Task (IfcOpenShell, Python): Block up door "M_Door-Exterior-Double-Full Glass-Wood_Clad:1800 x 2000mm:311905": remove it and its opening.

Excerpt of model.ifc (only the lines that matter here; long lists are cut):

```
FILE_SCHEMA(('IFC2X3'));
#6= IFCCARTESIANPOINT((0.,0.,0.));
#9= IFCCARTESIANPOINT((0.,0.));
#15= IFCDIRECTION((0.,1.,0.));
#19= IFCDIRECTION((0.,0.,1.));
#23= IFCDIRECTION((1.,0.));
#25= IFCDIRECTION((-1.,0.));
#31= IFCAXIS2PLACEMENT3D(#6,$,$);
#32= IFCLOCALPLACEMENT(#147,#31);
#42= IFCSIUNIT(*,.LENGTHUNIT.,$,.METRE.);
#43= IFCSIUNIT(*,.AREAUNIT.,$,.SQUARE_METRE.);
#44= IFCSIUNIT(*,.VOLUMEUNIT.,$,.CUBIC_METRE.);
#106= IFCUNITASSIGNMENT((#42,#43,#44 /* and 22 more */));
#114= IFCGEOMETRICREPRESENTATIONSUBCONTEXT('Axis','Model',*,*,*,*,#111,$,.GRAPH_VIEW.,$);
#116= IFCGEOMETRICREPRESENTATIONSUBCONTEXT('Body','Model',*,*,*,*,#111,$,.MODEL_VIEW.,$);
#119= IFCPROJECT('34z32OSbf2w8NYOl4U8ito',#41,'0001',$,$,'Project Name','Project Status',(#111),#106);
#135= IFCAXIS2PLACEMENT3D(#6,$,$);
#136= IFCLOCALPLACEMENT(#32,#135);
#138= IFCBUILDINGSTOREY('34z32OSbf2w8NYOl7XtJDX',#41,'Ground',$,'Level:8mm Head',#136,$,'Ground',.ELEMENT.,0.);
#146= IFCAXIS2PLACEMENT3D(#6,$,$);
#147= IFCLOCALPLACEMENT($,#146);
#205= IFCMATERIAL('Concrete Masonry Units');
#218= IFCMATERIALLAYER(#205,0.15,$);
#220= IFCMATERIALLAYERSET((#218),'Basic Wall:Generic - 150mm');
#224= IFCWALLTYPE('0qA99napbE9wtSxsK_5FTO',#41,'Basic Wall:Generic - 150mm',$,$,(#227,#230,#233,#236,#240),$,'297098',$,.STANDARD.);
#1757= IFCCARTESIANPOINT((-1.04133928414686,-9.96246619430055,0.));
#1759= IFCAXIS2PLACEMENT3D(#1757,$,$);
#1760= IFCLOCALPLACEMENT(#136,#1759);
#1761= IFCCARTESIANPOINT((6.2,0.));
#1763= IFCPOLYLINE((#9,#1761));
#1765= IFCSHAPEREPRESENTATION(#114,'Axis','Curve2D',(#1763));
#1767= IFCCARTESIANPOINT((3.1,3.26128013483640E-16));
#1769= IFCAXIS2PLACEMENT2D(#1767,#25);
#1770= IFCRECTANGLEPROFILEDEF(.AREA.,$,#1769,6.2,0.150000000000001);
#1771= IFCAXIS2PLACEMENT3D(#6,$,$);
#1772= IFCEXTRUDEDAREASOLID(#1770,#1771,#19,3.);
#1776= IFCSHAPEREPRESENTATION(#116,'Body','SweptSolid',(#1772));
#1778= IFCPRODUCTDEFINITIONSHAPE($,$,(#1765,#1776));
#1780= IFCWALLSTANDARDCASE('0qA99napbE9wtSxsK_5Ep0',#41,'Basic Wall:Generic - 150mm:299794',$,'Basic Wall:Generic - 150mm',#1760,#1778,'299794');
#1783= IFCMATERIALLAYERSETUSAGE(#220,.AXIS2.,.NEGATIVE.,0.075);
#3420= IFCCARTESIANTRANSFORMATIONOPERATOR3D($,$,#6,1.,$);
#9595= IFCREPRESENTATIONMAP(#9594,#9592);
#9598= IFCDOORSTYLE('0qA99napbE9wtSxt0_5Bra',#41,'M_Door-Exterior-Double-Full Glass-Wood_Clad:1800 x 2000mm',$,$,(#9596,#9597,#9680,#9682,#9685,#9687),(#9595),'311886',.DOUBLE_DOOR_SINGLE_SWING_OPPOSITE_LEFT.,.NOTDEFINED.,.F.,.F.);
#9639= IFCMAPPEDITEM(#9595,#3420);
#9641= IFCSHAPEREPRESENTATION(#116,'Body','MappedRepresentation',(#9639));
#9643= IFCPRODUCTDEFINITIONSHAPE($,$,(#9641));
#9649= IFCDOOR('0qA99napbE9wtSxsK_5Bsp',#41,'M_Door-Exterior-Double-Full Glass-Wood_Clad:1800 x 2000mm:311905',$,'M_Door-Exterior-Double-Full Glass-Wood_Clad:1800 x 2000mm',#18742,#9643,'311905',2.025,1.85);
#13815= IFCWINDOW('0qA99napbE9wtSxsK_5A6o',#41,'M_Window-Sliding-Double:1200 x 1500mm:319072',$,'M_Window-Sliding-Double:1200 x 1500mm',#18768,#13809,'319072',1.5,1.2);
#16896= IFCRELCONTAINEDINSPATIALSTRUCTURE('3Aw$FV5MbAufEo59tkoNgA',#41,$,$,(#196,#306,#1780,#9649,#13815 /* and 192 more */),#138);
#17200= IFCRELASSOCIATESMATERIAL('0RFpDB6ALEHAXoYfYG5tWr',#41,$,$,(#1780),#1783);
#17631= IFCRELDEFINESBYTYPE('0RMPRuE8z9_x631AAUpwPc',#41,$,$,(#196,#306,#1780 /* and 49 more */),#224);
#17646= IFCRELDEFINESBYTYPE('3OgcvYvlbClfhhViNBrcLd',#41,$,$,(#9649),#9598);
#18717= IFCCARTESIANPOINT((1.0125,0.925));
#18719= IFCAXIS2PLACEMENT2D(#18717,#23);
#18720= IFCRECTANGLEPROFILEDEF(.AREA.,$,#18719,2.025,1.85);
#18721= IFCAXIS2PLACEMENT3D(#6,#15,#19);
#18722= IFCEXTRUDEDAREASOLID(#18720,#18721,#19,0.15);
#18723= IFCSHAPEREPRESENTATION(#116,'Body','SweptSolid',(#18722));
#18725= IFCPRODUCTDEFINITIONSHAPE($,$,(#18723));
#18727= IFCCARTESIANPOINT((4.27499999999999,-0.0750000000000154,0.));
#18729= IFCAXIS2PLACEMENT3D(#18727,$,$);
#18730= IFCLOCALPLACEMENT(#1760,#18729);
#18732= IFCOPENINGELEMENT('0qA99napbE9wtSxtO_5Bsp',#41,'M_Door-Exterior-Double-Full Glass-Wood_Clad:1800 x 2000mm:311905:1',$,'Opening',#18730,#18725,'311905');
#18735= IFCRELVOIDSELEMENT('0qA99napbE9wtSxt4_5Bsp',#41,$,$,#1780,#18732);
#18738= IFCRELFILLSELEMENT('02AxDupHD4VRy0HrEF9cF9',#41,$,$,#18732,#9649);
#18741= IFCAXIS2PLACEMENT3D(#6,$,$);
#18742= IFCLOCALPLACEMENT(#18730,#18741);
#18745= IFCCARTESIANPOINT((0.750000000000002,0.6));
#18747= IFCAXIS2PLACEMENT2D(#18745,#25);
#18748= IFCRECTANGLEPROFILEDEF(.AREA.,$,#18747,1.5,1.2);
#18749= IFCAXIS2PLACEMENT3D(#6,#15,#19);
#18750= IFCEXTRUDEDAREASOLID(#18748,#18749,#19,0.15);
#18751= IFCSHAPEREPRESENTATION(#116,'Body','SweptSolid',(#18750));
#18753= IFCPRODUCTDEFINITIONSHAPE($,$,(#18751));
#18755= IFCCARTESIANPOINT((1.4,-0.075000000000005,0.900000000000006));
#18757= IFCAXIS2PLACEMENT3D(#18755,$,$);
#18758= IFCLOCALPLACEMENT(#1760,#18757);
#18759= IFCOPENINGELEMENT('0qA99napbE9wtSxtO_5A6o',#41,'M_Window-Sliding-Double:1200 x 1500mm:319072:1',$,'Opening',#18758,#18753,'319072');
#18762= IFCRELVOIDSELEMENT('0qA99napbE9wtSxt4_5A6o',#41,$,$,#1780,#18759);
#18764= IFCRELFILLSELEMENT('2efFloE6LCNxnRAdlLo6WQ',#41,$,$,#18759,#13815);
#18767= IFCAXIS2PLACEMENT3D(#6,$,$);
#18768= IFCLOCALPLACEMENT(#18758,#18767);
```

```python
import ifcopenshell
import ifcopenshell.api.feature
import ifcopenshell.api.root
import ifcopenshell.geom
import ifcopenshell.util.shape

model = ifcopenshell.open("model.ifc")
settings = ifcopenshell.geom.settings()


def volume(element):
    """Net volume in cubic metres, openings subtracted."""
    shape = ifcopenshell.geom.create_shape(settings, element)
    return ifcopenshell.util.shape.get_volume(shape.geometry)


door = model.by_guid("0qA99napbE9wtSxsK_5Bsp")
opening = door.FillsVoids[0].RelatingOpeningElement
wall = opening.VoidsElements[0].RelatingBuildingElement
before = volume(wall)

ifcopenshell.api.root.remove_product(model, product=door)
ifcopenshell.api.feature.remove_feature(model, feature=opening)

after = volume(wall)

print(f"wall volume {before:.3f} -> {after:.3f} m3")

model.write("model-out.ifc")
```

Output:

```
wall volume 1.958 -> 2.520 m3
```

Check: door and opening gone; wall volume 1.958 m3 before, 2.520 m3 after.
